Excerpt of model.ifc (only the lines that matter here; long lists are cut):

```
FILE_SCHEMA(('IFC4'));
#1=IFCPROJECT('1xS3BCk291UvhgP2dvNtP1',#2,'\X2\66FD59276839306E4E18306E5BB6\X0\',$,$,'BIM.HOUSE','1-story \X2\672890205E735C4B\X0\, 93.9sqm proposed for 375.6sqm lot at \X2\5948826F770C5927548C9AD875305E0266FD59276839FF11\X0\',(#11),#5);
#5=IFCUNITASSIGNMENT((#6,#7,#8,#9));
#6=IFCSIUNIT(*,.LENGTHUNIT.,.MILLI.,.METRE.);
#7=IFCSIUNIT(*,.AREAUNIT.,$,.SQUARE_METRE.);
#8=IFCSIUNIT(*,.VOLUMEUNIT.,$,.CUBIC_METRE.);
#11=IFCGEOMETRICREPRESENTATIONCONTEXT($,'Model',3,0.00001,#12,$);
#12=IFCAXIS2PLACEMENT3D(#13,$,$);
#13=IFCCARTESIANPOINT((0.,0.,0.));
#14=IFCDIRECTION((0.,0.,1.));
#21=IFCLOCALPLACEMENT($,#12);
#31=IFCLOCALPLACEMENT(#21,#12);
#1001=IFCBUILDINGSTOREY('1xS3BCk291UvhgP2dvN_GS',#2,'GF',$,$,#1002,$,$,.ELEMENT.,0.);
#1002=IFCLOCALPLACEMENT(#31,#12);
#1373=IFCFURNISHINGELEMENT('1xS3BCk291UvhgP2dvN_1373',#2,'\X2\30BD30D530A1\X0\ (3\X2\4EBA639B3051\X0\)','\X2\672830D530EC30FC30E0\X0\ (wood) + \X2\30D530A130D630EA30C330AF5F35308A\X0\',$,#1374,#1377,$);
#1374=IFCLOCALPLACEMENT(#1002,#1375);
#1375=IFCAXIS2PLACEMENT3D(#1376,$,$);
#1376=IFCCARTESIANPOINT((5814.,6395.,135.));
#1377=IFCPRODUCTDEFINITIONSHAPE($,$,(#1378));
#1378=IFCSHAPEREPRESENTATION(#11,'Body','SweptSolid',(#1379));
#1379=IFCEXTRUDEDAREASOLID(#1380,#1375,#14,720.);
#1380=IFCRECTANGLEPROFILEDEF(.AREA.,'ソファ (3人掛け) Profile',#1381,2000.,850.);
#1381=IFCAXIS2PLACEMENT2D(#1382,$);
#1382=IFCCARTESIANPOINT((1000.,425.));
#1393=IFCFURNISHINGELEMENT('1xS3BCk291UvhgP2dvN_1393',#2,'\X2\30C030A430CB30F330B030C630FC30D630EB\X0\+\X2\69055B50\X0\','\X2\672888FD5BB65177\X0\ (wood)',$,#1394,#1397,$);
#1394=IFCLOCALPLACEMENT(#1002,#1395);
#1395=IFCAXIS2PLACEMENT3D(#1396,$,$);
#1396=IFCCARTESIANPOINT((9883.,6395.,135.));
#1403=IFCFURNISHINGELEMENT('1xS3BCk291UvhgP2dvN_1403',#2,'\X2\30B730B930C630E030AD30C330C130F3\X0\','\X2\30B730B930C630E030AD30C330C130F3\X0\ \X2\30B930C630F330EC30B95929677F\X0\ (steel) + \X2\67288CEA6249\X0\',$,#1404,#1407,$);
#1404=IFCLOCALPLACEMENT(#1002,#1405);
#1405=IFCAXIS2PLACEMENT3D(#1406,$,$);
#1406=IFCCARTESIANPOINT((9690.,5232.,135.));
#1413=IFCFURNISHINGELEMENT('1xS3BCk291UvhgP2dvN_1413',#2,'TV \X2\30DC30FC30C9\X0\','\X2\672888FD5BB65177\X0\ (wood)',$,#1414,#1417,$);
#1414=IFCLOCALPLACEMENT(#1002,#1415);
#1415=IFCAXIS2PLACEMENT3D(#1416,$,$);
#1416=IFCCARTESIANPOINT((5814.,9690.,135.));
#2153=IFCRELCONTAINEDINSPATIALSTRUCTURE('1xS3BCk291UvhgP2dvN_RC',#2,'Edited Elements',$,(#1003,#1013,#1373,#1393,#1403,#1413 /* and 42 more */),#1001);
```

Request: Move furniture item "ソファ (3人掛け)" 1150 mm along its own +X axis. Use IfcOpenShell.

```python
import ifcopenshell
import ifcopenshell.api.geometry
import ifcopenshell.util.placement
import ifcopenshell.util.unit

model = ifcopenshell.open("model.ifc")
unit_scale = ifcopenshell.util.unit.calculate_unit_scale(model)

item = model.by_guid("1xS3BCk291UvhgP2dvN_1373")
matrix = ifcopenshell.util.placement.get_local_placement(item.ObjectPlacement)
matrix[:3, 3] += matrix[:3, 0] * 1.15 / unit_scale
ifcopenshell.api.geometry.edit_object_placement(model, product=item, matrix=matrix, is_si=False)

print(ifcopenshell.util.placement.get_local_placement(item.ObjectPlacement).round(3) + 0.0)

model.write("model_v2.ifc")
```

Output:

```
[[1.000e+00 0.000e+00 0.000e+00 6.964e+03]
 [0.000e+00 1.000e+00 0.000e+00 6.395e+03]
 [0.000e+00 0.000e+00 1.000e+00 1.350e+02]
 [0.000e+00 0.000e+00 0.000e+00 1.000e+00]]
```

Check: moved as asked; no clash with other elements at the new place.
